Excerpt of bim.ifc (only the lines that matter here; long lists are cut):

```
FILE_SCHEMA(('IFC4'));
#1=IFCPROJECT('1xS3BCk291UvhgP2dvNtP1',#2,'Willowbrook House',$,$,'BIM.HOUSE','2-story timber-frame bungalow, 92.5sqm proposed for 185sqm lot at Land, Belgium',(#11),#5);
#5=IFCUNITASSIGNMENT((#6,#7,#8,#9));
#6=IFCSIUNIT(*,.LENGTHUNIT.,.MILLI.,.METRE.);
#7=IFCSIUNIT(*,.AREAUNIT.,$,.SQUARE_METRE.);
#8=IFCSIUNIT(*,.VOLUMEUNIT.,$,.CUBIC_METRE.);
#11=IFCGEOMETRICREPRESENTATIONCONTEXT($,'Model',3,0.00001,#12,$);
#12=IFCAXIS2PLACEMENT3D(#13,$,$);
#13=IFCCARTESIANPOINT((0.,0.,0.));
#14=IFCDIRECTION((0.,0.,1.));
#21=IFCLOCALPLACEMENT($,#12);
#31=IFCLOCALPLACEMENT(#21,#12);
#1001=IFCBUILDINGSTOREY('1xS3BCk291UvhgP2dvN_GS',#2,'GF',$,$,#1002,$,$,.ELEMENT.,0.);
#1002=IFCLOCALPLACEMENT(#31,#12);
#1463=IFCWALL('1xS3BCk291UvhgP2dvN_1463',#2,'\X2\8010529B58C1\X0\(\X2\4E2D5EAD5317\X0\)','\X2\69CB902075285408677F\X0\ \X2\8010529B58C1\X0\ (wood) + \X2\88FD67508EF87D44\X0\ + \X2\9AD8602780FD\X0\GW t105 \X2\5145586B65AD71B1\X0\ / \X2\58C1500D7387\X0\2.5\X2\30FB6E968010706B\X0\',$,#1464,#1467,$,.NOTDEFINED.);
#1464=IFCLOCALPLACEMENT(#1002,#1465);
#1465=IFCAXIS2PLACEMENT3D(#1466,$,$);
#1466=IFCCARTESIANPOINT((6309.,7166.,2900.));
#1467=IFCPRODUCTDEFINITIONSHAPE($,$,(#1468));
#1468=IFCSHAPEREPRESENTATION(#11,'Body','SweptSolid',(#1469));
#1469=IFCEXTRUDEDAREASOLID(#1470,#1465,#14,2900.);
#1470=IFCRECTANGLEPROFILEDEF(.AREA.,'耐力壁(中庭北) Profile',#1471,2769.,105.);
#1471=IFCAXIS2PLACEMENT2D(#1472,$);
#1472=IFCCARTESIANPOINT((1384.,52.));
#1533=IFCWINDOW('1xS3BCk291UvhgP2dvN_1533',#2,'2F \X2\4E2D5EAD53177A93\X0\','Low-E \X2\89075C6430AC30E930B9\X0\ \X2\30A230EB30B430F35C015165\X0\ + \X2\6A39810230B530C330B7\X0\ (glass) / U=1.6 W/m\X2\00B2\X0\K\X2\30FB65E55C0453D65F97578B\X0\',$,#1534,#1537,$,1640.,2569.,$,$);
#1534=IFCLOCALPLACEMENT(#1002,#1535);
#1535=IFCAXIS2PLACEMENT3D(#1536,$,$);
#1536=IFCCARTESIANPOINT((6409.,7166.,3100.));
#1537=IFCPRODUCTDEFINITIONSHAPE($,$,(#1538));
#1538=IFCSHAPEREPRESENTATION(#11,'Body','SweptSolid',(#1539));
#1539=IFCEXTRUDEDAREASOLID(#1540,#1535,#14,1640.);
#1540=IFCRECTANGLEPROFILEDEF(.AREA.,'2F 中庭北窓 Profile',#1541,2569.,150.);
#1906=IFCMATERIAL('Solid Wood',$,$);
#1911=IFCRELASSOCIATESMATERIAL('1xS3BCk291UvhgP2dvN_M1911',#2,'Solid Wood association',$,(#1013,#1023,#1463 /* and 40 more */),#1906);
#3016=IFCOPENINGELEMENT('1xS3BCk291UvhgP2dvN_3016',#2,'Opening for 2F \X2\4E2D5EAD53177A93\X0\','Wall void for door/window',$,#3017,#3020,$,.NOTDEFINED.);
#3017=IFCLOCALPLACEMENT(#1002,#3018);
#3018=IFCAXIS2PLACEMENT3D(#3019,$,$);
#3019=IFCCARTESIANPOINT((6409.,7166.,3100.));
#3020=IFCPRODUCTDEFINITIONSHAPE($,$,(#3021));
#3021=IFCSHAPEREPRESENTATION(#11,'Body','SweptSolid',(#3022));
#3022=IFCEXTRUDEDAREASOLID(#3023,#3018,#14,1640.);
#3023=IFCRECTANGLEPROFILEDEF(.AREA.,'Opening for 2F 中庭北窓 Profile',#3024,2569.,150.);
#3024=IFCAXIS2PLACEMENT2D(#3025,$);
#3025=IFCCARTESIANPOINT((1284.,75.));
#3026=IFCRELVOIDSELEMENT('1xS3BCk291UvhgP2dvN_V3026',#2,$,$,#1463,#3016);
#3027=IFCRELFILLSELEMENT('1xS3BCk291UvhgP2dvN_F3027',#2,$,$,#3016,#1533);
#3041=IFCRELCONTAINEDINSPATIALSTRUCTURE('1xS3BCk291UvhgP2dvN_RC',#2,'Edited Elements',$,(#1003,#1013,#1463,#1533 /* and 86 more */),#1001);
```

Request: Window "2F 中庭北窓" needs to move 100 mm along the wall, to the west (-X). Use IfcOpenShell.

```python
import ifcopenshell
import ifcopenshell.api.geometry
import ifcopenshell.util.placement
import ifcopenshell.util.unit

model = ifcopenshell.open("bim.ifc")
unit_scale = ifcopenshell.util.unit.calculate_unit_scale(model)

window = model.by_guid("1xS3BCk291UvhgP2dvN_1533")
opening = window.FillsVoids[0].RelatingOpeningElement
wall = opening.VoidsElements[0].RelatingBuildingElement

wall_matrix = ifcopenshell.util.placement.get_local_placement(wall.ObjectPlacement)
shift = wall_matrix[:3, 0] * -0.1 / unit_scale
before = ifcopenshell.util.placement.get_local_placement(window.ObjectPlacement)[:3, 3].copy()

# The window is not placed relative to its opening, so move both.
for product in (opening, window):
    matrix = ifcopenshell.util.placement.get_local_placement(product.ObjectPlacement)
    matrix[:3, 3] += shift
    ifcopenshell.api.geometry.edit_object_placement(model, product=product, matrix=matrix, is_si=False)

after = ifcopenshell.util.placement.get_local_placement(window.ObjectPlacement)[:3, 3]
print("window moved by", (after - before).round(3) + 0.0)

model.write("bim_rev.ifc")
```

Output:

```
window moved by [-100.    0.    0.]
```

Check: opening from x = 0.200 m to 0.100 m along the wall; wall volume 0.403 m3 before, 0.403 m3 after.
